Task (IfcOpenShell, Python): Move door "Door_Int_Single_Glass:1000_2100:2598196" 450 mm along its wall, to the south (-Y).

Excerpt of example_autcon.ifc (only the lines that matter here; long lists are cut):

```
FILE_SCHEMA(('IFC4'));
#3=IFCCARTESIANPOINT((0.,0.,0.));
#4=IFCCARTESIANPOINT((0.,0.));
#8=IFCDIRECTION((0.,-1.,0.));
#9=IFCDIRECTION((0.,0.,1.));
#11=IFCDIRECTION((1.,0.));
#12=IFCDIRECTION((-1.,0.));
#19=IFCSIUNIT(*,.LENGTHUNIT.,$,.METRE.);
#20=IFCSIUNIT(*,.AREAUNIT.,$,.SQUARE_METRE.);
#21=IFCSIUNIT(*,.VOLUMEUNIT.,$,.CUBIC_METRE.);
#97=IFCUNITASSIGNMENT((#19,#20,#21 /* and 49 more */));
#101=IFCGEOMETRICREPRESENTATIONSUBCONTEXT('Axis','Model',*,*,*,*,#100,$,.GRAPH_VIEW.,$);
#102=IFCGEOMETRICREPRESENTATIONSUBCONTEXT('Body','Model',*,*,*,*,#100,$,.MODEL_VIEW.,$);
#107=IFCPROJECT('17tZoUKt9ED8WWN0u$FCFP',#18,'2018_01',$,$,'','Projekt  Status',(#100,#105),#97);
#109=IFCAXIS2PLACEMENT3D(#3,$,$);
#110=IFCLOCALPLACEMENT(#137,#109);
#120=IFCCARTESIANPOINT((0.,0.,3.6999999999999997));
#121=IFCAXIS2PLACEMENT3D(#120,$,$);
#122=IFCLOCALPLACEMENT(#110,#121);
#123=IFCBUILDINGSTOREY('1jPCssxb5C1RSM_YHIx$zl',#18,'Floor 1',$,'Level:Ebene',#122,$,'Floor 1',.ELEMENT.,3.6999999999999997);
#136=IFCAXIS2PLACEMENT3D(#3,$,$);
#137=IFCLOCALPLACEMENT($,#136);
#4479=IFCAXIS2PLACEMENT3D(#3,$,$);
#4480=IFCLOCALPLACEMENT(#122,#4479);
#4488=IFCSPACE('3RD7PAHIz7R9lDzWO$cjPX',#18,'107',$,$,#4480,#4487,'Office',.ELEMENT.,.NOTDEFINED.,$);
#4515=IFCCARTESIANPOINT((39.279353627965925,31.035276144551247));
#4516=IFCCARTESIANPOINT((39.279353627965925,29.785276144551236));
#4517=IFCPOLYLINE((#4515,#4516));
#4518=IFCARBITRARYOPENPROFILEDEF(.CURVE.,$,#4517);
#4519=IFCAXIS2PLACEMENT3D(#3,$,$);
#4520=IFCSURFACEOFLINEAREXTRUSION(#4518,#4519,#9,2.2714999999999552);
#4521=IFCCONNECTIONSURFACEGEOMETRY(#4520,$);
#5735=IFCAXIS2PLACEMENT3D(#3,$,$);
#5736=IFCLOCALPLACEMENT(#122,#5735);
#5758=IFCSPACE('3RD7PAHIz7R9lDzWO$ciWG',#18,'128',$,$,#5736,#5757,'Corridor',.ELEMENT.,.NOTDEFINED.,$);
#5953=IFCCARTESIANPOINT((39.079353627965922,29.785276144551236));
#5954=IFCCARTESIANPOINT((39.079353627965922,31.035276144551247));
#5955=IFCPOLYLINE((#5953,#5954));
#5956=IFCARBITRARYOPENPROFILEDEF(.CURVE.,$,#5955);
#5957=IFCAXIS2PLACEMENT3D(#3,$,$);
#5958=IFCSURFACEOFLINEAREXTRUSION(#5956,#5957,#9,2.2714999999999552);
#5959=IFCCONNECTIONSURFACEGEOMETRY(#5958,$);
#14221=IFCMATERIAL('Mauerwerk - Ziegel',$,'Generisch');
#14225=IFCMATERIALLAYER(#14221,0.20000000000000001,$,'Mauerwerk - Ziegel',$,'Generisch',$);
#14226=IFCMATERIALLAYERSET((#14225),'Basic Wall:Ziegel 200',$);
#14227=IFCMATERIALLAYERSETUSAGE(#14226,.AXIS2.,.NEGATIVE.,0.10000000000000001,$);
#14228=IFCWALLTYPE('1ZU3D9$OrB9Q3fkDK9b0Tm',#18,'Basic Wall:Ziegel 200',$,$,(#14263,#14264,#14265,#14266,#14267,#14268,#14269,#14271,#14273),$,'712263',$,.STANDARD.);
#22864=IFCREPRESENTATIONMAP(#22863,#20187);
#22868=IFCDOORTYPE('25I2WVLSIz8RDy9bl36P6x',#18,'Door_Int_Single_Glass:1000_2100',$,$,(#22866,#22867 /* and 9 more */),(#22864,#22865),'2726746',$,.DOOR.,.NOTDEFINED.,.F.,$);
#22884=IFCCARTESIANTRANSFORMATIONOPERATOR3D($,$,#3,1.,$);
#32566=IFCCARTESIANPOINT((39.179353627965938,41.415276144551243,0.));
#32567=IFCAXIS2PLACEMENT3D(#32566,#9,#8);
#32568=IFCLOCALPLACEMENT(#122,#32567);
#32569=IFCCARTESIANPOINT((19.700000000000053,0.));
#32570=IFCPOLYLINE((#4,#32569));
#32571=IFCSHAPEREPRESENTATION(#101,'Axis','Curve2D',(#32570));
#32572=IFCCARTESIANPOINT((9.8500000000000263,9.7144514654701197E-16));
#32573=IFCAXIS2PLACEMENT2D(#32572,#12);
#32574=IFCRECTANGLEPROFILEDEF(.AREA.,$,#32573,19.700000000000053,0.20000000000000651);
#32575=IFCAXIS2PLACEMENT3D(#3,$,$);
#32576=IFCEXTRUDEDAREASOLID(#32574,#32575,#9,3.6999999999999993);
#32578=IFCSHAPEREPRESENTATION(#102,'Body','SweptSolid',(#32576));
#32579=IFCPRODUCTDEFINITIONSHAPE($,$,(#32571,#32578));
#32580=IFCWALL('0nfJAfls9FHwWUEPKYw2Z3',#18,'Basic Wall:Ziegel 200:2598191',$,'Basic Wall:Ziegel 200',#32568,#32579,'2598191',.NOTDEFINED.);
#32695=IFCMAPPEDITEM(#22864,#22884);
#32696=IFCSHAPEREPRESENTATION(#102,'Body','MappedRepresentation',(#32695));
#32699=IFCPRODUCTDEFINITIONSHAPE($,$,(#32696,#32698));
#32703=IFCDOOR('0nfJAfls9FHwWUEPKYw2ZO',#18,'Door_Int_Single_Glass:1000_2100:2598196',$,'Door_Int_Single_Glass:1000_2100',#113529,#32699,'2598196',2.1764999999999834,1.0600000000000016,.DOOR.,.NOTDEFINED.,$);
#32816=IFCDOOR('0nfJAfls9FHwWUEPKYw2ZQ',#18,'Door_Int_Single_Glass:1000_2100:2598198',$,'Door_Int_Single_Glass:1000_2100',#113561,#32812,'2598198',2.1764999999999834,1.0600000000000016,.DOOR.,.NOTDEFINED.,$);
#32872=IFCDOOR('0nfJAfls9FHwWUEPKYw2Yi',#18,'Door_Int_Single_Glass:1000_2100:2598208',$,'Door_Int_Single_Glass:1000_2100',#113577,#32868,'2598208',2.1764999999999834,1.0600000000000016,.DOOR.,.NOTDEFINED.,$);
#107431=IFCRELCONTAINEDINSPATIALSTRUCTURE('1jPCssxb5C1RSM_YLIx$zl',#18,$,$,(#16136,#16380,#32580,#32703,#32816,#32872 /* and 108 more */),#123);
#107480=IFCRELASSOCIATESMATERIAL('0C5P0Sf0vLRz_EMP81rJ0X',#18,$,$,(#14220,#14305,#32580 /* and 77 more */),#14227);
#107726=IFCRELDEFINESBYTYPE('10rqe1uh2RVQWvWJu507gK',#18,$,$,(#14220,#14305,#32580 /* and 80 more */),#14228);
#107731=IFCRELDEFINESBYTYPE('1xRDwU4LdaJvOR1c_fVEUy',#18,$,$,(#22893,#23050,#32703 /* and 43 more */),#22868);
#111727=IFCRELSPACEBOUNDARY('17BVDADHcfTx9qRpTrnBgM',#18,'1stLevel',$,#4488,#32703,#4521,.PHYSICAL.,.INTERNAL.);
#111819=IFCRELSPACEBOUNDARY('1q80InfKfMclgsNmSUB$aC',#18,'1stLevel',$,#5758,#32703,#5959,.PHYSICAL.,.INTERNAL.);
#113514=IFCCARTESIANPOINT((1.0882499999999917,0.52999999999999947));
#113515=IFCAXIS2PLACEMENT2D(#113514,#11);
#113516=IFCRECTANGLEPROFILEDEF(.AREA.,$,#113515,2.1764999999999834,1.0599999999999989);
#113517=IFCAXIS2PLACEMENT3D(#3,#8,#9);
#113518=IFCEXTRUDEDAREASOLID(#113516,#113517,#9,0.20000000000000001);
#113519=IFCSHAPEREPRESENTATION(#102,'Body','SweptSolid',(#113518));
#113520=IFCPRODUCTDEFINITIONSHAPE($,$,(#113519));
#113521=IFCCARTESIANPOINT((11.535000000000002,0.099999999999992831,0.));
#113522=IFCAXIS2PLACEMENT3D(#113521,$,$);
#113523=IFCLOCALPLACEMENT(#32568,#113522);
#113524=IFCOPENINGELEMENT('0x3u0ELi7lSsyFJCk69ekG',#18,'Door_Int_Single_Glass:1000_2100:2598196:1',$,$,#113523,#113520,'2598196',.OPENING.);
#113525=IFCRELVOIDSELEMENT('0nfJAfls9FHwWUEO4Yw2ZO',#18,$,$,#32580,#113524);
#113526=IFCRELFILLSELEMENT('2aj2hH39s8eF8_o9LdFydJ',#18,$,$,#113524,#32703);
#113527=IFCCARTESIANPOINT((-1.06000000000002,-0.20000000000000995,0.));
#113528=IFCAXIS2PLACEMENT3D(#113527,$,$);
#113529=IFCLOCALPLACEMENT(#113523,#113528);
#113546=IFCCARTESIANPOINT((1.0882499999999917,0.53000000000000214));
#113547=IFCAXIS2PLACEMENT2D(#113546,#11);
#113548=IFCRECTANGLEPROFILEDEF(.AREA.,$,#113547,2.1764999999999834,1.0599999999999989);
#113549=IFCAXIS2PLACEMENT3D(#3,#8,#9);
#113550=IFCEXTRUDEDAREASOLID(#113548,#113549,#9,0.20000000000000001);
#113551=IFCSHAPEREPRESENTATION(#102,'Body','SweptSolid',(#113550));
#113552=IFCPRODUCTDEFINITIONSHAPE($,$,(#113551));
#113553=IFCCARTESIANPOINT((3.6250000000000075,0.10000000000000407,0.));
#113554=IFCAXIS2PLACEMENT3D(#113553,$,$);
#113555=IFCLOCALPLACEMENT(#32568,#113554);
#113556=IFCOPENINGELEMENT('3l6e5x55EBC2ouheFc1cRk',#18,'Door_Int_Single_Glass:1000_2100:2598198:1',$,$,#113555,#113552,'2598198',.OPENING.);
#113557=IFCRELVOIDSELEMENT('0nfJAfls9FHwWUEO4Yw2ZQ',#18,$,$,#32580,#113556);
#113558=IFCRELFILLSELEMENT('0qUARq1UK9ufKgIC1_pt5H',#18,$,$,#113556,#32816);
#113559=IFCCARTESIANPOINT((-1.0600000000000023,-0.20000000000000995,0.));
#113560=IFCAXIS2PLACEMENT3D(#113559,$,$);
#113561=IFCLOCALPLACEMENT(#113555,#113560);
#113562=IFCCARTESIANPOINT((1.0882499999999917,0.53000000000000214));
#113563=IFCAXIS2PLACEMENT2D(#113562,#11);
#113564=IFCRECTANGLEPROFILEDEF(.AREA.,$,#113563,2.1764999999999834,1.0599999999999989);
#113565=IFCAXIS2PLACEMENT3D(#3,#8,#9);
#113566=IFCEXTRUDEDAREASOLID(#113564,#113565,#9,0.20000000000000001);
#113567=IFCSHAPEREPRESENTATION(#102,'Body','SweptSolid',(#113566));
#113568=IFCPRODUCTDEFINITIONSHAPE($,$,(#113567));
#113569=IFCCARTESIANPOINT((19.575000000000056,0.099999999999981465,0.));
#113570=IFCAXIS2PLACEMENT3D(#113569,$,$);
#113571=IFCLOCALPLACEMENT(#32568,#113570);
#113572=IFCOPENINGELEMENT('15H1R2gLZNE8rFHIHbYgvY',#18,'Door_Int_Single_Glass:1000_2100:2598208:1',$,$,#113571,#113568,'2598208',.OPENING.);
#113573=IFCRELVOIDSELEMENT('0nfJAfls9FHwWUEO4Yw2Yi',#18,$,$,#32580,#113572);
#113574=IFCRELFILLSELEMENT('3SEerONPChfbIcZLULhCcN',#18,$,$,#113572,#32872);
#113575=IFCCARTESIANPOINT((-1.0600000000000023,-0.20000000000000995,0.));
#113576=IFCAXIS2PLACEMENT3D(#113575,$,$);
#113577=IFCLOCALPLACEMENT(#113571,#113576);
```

```python
import numpy as np
import ifcopenshell
import ifcopenshell.api.geometry
import ifcopenshell.util.placement
import ifcopenshell.util.unit

model = ifcopenshell.open("example_autcon.ifc")
unit_scale = ifcopenshell.util.unit.calculate_unit_scale(model)

door = model.by_guid("0nfJAfls9FHwWUEPKYw2ZO")
opening = door.FillsVoids[0].RelatingOpeningElement
wall = opening.VoidsElements[0].RelatingBuildingElement

wall_matrix = ifcopenshell.util.placement.get_local_placement(wall.ObjectPlacement)
shift = wall_matrix[:3, 0] * 0.45 / unit_scale
before = ifcopenshell.util.placement.get_local_placement(door.ObjectPlacement)[:3, 3].copy()

# The door is placed relative to its opening, so it follows when the opening moves.
matrix = ifcopenshell.util.placement.get_local_placement(opening.ObjectPlacement)
matrix[:3, 3] += shift
ifcopenshell.api.geometry.edit_object_placement(
    model, product=opening, matrix=matrix, is_si=False, should_transform_children=True
)

# Space boundary surfaces are stored in each space's coordinates; move them too.
for rel in door.ProvidesBoundaries:
    if not rel.ConnectionGeometry:
        continue
    surface = rel.ConnectionGeometry.SurfaceOnRelatingElement
    space_matrix = ifcopenshell.util.placement.get_local_placement(rel.RelatingSpace.ObjectPlacement)
    point = np.array(surface.Position.Location.Coordinates) + space_matrix[:3, :3].T @ shift
    surface.Position = model.createIfcAxis2Placement3D(
        model.createIfcCartesianPoint(point.tolist()), surface.Position.Axis, surface.Position.RefDirection
    )

after = ifcopenshell.util.placement.get_local_placement(door.ObjectPlacement)[:3, 3]
print("door moved by", (after - before).round(3) + 0.0)

model.write("example_autcon_edited.ifc")
```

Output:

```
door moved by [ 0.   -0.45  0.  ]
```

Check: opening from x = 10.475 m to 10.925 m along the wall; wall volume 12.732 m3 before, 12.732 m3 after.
